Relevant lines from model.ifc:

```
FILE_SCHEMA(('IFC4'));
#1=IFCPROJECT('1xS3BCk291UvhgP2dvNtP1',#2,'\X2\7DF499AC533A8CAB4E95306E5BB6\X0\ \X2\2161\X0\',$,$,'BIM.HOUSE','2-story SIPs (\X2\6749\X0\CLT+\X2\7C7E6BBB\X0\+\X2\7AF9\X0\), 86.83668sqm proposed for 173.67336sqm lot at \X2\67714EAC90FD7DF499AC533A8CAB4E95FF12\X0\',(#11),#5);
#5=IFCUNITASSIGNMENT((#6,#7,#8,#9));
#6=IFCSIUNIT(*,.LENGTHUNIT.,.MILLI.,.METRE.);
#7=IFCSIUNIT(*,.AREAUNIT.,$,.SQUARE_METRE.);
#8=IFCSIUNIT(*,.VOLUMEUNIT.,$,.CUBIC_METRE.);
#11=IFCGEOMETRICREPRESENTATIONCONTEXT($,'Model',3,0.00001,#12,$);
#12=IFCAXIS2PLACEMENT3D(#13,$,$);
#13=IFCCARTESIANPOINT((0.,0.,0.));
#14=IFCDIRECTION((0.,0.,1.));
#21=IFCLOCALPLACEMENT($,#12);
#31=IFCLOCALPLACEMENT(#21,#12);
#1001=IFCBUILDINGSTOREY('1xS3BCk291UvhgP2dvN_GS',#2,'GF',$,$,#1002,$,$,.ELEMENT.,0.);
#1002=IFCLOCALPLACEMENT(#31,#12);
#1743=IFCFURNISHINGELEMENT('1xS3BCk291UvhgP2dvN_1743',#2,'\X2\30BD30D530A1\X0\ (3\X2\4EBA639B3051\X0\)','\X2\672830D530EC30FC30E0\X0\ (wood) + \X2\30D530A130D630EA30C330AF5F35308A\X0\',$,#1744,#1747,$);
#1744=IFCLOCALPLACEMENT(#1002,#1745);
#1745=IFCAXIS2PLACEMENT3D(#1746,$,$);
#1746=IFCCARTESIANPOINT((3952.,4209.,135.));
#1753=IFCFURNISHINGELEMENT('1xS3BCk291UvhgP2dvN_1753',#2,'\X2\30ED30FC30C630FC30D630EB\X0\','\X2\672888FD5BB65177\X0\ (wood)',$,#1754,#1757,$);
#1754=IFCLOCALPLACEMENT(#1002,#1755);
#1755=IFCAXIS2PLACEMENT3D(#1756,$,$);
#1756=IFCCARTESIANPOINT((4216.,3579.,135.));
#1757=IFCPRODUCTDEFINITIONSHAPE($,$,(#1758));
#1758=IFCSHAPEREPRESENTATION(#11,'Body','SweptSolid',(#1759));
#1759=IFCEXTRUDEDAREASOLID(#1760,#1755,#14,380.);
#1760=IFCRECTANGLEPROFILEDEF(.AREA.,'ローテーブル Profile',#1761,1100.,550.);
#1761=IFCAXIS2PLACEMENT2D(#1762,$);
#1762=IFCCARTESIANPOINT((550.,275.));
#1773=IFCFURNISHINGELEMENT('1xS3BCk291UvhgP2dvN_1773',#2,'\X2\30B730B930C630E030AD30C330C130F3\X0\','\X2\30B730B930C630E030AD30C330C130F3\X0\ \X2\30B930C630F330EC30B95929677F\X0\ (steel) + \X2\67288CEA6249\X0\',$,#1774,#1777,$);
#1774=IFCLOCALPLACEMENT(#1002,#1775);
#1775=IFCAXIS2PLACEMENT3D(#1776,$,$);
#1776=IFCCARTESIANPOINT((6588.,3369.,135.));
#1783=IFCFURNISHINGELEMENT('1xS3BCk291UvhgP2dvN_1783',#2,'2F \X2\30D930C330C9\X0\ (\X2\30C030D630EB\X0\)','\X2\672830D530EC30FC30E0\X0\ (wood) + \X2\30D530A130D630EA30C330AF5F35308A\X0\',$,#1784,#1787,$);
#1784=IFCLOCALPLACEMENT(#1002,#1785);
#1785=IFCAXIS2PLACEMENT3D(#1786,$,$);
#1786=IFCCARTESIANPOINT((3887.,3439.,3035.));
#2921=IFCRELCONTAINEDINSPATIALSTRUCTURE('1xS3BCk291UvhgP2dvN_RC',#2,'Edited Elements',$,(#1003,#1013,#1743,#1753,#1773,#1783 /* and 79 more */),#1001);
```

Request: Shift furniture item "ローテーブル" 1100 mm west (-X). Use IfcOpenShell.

```python
import ifcopenshell
import ifcopenshell.api.geometry
import ifcopenshell.util.placement

model = ifcopenshell.open("model.ifc")

item = model.by_guid("1xS3BCk291UvhgP2dvN_1753")
matrix = ifcopenshell.util.placement.get_local_placement(item.ObjectPlacement)
matrix[0, 3] -= 1100.0
ifcopenshell.api.geometry.edit_object_placement(model, product=item, matrix=matrix, is_si=False)

print(ifcopenshell.util.placement.get_local_placement(item.ObjectPlacement).round(3) + 0.0)

model.write("model_updated.ifc")
```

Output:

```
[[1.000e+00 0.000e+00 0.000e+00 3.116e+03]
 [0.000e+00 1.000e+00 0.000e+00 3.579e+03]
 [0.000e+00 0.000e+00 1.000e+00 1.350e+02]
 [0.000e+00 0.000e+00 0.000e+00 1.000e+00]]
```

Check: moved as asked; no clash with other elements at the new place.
